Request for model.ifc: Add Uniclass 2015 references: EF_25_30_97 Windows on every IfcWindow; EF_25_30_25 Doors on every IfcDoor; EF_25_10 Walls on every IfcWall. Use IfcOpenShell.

First a look at what the model holds.

```python
import ifcopenshell

model = ifcopenshell.open("model.ifc")
print(model.schema)
print("classifications:", [c.Name for c in model.by_type("IfcClassification")])
for ifc_class in ("IfcDoor", "IfcRoof", "IfcStair", "IfcWall", "IfcWindow"):
    print(ifc_class, len(model.by_type(ifc_class)))
```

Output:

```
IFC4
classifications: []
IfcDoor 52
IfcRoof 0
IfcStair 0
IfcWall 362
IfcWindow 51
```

```python
import ifcopenshell
import ifcopenshell.api.classification

model = ifcopenshell.open("model.ifc")

system = ifcopenshell.api.classification.add_classification(model, classification="Uniclass 2015")

codes = {
    "IfcWindow": ("EF_25_30_97", "Windows"),
    "IfcDoor": ("EF_25_30_25", "Doors"),
    "IfcWall": ("EF_25_10", "Walls"),
}
for ifc_class, (code, name) in codes.items():
    products = model.by_type(ifc_class)
    ifcopenshell.api.classification.add_reference(
        model, products=products, classification=system, identification=code, name=name
    )
    print(code, len(products))

model.write("model_rev.ifc")
```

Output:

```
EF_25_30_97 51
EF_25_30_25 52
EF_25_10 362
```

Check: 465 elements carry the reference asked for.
